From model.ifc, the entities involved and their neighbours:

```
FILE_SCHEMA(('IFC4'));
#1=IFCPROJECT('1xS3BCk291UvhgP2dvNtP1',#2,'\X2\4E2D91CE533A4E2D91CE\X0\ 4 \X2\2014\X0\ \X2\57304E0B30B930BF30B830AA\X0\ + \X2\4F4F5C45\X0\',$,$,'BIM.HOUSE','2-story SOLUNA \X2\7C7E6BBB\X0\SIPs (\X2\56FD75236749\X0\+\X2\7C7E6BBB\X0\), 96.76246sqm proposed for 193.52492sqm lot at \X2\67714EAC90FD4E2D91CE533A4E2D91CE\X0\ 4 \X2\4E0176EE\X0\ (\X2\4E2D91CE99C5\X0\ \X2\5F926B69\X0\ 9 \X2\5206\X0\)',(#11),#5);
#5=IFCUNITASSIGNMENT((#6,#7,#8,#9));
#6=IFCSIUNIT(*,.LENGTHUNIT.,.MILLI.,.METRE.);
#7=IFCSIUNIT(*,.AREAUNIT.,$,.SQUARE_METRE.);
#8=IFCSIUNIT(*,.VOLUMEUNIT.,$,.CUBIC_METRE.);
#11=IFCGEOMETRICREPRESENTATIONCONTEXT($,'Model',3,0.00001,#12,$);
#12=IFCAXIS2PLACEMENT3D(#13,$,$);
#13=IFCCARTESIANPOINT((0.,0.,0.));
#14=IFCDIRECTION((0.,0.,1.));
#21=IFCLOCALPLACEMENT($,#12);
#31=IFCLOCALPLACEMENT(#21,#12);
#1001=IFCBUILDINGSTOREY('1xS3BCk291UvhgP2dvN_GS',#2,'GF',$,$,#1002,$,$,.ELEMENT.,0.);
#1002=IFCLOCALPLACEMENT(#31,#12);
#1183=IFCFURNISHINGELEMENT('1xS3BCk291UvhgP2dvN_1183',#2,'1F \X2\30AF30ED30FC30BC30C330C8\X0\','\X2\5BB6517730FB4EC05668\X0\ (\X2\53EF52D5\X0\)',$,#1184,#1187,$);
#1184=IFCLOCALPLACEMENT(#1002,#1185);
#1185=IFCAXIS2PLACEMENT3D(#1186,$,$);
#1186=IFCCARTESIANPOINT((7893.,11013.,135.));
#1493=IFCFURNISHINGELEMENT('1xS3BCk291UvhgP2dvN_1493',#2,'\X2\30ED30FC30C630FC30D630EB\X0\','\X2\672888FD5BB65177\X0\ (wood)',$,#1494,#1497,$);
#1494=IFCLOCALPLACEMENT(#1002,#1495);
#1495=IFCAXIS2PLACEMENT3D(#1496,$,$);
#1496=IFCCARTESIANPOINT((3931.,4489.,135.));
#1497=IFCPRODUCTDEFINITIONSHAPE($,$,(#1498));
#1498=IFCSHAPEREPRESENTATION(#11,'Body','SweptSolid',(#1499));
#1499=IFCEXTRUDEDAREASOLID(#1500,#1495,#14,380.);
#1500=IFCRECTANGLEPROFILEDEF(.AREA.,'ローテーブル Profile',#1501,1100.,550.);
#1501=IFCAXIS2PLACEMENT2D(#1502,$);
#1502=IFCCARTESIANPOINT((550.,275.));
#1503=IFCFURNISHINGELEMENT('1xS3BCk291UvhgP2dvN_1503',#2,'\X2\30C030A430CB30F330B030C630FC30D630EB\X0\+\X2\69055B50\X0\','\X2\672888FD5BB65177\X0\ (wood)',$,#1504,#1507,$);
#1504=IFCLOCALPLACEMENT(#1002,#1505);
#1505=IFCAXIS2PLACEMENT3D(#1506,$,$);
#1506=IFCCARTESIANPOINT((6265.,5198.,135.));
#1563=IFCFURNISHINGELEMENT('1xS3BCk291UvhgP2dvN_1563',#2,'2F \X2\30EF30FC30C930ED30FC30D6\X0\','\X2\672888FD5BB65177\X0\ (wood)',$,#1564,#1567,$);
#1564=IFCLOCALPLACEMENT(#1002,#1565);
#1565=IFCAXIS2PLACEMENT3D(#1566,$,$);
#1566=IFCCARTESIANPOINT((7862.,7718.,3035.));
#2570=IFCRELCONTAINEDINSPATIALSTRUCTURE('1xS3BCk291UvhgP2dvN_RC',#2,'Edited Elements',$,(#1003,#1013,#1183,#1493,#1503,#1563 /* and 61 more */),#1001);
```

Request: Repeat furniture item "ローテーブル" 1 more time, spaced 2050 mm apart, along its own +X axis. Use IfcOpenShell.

```python
import ifcopenshell
import ifcopenshell.api.geometry
import ifcopenshell.api.root
import ifcopenshell.util.element
import ifcopenshell.util.placement
import ifcopenshell.util.unit

model = ifcopenshell.open("model.ifc")
unit_scale = ifcopenshell.util.unit.calculate_unit_scale(model)


def reuse_history(source, copy):
    """copy_class also copies each property set's owner history, people and application; keep the originals."""
    for rel in copy.IsDefinedBy:
        if rel.is_a("IfcRelDefinesByProperties") and (history := rel.RelatingPropertyDefinition.OwnerHistory):
            rel.RelatingPropertyDefinition.OwnerHistory = source.OwnerHistory
            ifcopenshell.util.element.remove_deep2(model, history)


source = model.by_guid("1xS3BCk291UvhgP2dvN_1493")
base = ifcopenshell.util.placement.get_local_placement(source.ObjectPlacement)
step = base[:3, 0] * 2.05 / unit_scale

for i in range(1, 2):
    copy = ifcopenshell.api.root.copy_class(model, product=source)
    copy.Representation = ifcopenshell.util.element.copy_deep(
        model, source.Representation, exclude=["IfcGeometricRepresentationContext", "IfcRepresentationMap"]
    )
    reuse_history(source, copy)
    matrix = base.copy()
    matrix[:3, 3] += i * step
    print("added at", matrix[:3, 3].round(3) + 0.0)
    ifcopenshell.api.geometry.edit_object_placement(model, product=copy, matrix=matrix, is_si=False)

model.write("model_updated.ifc")
```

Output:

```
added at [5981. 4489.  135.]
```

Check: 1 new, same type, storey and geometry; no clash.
